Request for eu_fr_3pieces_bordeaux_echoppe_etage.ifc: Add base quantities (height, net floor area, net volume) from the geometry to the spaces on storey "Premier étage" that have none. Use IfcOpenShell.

First a look at what the model holds.

```python
import ifcopenshell
import ifcopenshell.util.element
import ifcopenshell.util.unit

model = ifcopenshell.open("eu_fr_3pieces_bordeaux_echoppe_etage.ifc")
print(model.schema)
for unit_type in ("LENGTHUNIT", "AREAUNIT", "VOLUMEUNIT"):
    print(unit_type, ifcopenshell.util.unit.calculate_unit_scale(model, unit_type))
storey = next(s for s in model.by_type("IfcBuildingStorey") if s.Name == "Premier étage")
spaces = [e for e in ifcopenshell.util.element.get_decomposition(storey) if e.is_a("IfcSpace")]
for e in sorted(spaces, key=lambda e: e.id()):
    print(e.id(), e.is_a(), e.Name, list(ifcopenshell.util.element.get_psets(e, qtos_only=True)), sep=" | ")
```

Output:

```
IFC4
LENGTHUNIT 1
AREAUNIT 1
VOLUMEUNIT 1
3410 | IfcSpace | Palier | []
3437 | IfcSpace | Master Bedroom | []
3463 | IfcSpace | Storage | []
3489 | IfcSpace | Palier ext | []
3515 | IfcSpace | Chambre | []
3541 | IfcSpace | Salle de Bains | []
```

```python
import ifcopenshell
import ifcopenshell.api.pset
import ifcopenshell.geom
import ifcopenshell.util.element
import ifcopenshell.util.shape
import ifcopenshell.util.unit

model = ifcopenshell.open("eu_fr_3pieces_bordeaux_echoppe_etage.ifc")
unit_scale = ifcopenshell.util.unit.calculate_unit_scale(model)
area_scale = ifcopenshell.util.unit.calculate_unit_scale(model, "AREAUNIT")
volume_scale = ifcopenshell.util.unit.calculate_unit_scale(model, "VOLUMEUNIT")
settings = ifcopenshell.geom.settings()

storey = next(s for s in model.by_type("IfcBuildingStorey") if s.Name == "Premier étage")
spaces = [e for e in ifcopenshell.util.element.get_decomposition(storey) if e.is_a("IfcSpace")]

for e in sorted(spaces, key=lambda e: e.id()):
    if ifcopenshell.util.element.get_psets(e, qtos_only=True, should_inherit=False):
        continue
    # Geometry comes back in metres, in the element's own axes.
    shape = ifcopenshell.geom.create_shape(settings, e)
    values = {
        "Height": ifcopenshell.util.shape.get_z(shape.geometry) / unit_scale,
        "NetFloorArea": ifcopenshell.util.shape.get_footprint_area(shape.geometry) / area_scale,
        "NetVolume": ifcopenshell.util.shape.get_volume(shape.geometry) / volume_scale,
    }
    qto = ifcopenshell.api.pset.add_qto(model, product=e, name="Qto_SpaceBaseQuantities")
    ifcopenshell.api.pset.edit_qto(model, qto=qto, properties=values)
    print(e.id(), {k: round(v, 3) for k, v in values.items()})

model.write("eu_fr_3pieces_bordeaux_echoppe_etage-out.ifc")
```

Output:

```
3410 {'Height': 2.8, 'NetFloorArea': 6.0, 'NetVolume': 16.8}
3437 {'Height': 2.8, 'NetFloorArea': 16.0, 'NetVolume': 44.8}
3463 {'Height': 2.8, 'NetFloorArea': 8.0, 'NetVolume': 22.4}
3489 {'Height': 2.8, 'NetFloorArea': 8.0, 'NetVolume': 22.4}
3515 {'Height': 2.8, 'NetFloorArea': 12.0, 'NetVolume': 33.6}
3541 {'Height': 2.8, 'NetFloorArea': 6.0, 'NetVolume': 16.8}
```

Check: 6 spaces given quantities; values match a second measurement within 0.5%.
